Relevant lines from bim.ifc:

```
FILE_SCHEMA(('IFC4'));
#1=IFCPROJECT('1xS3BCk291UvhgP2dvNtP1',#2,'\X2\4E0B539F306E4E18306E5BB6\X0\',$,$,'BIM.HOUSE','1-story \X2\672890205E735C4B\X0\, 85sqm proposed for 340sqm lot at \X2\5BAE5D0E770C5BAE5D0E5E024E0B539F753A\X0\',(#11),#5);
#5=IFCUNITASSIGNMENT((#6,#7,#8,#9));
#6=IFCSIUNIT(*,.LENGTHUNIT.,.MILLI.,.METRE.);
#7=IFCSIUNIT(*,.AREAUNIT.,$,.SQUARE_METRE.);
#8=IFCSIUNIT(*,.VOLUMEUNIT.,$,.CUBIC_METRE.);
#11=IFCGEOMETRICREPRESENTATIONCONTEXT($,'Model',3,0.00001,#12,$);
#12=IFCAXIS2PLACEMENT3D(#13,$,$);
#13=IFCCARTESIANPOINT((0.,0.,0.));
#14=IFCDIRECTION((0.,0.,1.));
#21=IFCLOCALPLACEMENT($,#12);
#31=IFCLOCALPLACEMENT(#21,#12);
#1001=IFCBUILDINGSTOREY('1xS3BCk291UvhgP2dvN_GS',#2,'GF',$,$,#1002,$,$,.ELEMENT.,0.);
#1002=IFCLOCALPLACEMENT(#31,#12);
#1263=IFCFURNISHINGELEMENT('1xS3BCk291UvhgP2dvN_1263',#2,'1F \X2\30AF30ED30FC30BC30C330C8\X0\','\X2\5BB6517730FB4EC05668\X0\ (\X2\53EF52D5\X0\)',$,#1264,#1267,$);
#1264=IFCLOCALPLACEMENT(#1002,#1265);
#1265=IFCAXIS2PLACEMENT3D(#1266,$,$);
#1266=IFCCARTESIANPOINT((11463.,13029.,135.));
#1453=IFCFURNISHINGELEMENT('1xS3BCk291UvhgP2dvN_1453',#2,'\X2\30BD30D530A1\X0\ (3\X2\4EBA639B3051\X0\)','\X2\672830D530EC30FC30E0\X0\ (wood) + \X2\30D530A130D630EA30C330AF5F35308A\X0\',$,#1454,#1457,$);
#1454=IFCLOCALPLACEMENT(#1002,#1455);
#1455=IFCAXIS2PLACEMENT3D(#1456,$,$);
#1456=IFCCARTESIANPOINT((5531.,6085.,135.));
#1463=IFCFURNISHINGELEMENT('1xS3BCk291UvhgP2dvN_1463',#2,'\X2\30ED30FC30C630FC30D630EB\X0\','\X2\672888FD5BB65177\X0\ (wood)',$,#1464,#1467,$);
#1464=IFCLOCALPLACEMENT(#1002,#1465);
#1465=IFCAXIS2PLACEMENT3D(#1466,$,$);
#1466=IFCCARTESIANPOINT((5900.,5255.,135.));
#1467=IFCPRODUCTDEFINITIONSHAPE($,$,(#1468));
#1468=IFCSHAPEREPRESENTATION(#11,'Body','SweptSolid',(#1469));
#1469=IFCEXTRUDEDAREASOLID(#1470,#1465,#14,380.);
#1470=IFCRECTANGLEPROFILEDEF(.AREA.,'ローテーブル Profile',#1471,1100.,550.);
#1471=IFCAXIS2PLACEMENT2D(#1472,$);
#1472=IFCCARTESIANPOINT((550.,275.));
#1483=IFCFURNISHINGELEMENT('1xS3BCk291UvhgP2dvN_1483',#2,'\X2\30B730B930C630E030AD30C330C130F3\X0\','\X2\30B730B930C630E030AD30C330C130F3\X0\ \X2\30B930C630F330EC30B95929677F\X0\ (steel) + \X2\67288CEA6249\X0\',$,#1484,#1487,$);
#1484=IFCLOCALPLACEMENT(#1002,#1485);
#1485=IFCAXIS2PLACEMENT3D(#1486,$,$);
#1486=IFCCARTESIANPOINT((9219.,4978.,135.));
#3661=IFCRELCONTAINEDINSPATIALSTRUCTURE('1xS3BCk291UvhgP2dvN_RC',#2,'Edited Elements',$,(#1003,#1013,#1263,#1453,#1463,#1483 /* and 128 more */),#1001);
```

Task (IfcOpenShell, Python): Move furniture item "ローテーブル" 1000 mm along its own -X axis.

```python
import ifcopenshell
import ifcopenshell.api.geometry
import ifcopenshell.util.placement

model = ifcopenshell.open("bim.ifc")

item = model.by_guid("1xS3BCk291UvhgP2dvN_1463")
matrix = ifcopenshell.util.placement.get_local_placement(item.ObjectPlacement)
matrix[:3, 3] -= matrix[:3, 0] * 1000.0
ifcopenshell.api.geometry.edit_object_placement(model, product=item, matrix=matrix, is_si=False)

print(ifcopenshell.util.placement.get_local_placement(item.ObjectPlacement).round(3) + 0.0)

model.write("bim_rev.ifc")
```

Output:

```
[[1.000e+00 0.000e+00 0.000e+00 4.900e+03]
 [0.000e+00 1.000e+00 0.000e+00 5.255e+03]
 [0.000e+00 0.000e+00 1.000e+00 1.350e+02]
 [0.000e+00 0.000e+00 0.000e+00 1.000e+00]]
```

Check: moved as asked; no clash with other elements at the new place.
